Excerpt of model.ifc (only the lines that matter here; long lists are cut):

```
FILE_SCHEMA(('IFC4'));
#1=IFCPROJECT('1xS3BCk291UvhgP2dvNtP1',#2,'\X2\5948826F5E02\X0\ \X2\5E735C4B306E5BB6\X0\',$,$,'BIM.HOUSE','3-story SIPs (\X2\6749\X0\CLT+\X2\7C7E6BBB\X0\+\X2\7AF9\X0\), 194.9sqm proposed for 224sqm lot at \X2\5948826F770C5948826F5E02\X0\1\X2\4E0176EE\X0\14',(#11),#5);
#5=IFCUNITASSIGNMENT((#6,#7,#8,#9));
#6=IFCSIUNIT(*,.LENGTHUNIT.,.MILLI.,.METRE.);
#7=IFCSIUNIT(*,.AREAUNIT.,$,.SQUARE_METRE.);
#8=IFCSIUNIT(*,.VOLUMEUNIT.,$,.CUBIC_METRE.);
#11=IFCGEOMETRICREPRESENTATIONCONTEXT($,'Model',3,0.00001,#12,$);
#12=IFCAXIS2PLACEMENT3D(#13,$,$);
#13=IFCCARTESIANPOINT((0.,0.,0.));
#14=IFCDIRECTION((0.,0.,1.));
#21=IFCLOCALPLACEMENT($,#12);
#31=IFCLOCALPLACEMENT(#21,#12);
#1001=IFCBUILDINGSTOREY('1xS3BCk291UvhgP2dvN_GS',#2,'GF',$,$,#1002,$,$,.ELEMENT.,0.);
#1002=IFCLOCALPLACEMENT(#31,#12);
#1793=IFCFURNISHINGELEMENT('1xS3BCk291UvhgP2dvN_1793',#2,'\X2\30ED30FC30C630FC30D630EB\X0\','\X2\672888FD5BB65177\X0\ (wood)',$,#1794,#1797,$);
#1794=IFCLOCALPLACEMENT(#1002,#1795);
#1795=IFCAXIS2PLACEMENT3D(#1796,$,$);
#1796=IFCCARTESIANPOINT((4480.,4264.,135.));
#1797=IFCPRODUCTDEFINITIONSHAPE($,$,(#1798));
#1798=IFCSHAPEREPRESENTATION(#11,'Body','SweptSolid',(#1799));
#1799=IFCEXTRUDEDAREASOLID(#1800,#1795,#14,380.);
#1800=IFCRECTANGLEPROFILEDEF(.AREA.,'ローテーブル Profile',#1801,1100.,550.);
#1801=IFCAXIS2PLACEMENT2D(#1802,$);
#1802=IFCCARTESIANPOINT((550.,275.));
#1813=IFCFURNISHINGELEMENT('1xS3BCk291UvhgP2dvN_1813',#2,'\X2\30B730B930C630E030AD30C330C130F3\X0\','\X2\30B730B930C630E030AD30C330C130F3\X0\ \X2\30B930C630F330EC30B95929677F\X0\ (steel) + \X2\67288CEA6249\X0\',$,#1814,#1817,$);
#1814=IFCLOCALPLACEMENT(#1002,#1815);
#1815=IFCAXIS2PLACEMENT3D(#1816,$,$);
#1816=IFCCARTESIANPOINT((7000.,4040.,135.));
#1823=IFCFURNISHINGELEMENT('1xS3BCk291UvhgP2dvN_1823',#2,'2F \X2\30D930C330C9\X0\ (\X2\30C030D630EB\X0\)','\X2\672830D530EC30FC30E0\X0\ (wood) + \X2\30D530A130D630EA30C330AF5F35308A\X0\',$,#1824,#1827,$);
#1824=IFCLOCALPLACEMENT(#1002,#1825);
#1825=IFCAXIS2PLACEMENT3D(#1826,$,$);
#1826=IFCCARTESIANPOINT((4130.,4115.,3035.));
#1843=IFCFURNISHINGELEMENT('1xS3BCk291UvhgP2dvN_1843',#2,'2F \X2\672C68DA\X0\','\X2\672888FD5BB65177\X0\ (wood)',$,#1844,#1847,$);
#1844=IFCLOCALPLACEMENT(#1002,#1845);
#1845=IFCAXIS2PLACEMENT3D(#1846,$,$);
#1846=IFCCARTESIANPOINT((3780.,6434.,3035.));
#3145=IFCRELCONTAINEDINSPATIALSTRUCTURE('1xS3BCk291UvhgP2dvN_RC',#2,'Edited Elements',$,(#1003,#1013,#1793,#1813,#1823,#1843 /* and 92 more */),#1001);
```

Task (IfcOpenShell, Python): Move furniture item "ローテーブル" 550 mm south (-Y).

```python
import ifcopenshell
import ifcopenshell.api.geometry
import ifcopenshell.util.placement
import ifcopenshell.util.unit

model = ifcopenshell.open("model.ifc")
unit_scale = ifcopenshell.util.unit.calculate_unit_scale(model)

item = model.by_guid("1xS3BCk291UvhgP2dvN_1793")
matrix = ifcopenshell.util.placement.get_local_placement(item.ObjectPlacement)
matrix[1, 3] -= 0.55 / unit_scale
ifcopenshell.api.geometry.edit_object_placement(model, product=item, matrix=matrix, is_si=False)

print(ifcopenshell.util.placement.get_local_placement(item.ObjectPlacement).round(3) + 0.0)

model.write("model_updated.ifc")
```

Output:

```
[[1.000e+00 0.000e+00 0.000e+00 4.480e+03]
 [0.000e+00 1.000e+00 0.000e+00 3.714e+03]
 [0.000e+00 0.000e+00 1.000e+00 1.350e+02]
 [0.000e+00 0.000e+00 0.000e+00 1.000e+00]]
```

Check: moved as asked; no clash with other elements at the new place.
